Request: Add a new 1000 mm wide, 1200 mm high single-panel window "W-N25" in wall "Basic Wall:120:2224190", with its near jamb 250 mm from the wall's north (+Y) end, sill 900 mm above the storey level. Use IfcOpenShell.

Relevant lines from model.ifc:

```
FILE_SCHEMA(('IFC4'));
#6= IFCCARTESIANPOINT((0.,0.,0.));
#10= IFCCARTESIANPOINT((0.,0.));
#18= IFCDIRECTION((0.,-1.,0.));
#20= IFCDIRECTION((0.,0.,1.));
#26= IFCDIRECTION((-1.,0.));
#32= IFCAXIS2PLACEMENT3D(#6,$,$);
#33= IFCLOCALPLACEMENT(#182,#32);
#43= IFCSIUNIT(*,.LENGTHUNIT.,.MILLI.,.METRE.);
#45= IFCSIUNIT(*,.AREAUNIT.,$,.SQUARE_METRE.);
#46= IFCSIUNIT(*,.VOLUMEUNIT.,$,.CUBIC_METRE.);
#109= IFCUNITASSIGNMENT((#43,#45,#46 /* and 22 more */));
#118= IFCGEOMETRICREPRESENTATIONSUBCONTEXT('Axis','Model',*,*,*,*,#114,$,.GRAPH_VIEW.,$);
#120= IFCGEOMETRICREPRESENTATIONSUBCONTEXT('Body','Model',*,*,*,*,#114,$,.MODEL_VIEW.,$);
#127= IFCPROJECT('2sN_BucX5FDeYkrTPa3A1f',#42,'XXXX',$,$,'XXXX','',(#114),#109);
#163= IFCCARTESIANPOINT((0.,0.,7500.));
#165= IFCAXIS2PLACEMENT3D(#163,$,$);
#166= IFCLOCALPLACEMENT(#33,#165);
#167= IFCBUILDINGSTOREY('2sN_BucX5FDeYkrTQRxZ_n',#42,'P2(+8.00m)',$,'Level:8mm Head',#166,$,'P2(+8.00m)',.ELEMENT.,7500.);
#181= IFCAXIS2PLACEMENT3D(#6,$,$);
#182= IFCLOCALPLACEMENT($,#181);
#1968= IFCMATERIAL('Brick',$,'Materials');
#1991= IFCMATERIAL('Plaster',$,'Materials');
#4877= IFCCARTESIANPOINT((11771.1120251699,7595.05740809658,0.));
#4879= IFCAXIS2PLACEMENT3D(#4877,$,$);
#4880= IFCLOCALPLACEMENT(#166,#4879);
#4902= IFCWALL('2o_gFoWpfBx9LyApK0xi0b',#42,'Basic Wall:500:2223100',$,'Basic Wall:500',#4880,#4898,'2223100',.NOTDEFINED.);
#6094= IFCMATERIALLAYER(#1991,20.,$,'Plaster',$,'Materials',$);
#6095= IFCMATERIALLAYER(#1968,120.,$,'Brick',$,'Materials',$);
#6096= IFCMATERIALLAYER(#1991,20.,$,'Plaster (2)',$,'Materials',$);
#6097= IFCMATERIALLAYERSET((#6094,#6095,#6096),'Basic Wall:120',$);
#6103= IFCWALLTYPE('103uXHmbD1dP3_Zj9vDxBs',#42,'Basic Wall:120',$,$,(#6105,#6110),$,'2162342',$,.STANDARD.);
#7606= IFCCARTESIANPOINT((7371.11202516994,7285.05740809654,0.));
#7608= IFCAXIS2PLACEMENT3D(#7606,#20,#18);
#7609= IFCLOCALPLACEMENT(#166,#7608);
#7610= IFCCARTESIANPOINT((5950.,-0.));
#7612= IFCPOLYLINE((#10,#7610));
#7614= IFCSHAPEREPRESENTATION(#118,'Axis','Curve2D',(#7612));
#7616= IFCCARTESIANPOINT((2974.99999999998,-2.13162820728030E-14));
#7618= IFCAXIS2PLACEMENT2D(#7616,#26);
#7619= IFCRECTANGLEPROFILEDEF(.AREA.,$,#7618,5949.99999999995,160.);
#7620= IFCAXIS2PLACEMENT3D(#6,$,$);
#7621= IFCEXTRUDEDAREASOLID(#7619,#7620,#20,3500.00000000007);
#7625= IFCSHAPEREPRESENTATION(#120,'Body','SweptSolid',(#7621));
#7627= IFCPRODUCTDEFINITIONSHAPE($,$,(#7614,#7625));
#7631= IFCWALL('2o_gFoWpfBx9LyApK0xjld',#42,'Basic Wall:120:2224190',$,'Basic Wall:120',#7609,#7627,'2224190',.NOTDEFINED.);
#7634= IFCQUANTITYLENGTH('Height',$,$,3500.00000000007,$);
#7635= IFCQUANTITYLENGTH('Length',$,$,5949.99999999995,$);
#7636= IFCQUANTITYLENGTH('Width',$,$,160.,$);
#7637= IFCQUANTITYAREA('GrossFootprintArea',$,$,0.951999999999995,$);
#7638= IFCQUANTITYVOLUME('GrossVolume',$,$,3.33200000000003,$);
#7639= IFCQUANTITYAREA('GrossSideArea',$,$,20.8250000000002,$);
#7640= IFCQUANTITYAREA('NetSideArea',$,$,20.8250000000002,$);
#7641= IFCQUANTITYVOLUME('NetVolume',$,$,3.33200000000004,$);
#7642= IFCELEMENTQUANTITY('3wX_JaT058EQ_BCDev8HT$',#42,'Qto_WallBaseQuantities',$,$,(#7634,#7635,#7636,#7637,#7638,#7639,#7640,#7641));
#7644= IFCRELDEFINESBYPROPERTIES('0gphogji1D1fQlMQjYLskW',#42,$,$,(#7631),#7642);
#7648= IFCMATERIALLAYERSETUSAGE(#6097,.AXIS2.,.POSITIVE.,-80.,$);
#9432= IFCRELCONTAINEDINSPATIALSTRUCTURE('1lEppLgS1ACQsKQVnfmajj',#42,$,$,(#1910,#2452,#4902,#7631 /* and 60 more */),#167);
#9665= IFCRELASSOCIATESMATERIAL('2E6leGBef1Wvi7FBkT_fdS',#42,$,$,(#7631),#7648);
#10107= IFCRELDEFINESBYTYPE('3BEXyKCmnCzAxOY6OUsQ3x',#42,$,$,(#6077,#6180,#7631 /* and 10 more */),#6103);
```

```python
import numpy as np
import ifcopenshell
import ifcopenshell.api.feature
import ifcopenshell.api.geometry
import ifcopenshell.api.pset
import ifcopenshell.api.root
import ifcopenshell.api.spatial
import ifcopenshell.geom
import ifcopenshell.util.element
import ifcopenshell.util.placement
import ifcopenshell.util.representation
import ifcopenshell.util.shape
import ifcopenshell.util.unit

model = ifcopenshell.open("model.ifc")
unit_scale = ifcopenshell.util.unit.calculate_unit_scale(model)
area_scale = ifcopenshell.util.unit.calculate_unit_scale(model, "AREAUNIT")
volume_scale = ifcopenshell.util.unit.calculate_unit_scale(model, "VOLUMEUNIT")
settings = ifcopenshell.geom.settings()


def volume(element):
    """Net volume in cubic metres, openings subtracted."""
    shape = ifcopenshell.geom.create_shape(settings, element)
    return ifcopenshell.util.shape.get_volume(shape.geometry)


wall = model.by_guid("2o_gFoWpfBx9LyApK0xjld")
storey = ifcopenshell.util.element.get_container(wall, ifc_class="IfcBuildingStorey")
context = ifcopenshell.util.representation.get_context(model, "Model", "Body", "MODEL_VIEW")
before = volume(wall)

width, height, from_end, sill = 1, 1.2, 0.25, 0.9  # metres

# The wall runs along its own X axis, and the end named is its -X end.
wall_shape = ifcopenshell.geom.create_shape(settings, wall)
x, y, z = ifcopenshell.util.shape.get_vertices(wall_shape.geometry).T
start = x.min() + from_end
face, thickness = float(y.min()), float(y.max() - y.min())
wall_matrix = ifcopenshell.util.placement.get_local_placement(wall.ObjectPlacement)
level = ifcopenshell.util.placement.get_local_placement(storey.ObjectPlacement)[2, 3]


def in_wall(x, y):
    """Placement at x, y metres in the wall's axes, at sill height."""
    matrix = wall_matrix.copy()
    matrix[:, 3] = wall_matrix @ np.array([x / unit_scale, y / unit_scale, 0.0, 1.0])
    matrix[2, 3] = level + sill / unit_scale
    return matrix


# Opening: a box that overshoots both wall faces by 50 mm.
opening = ifcopenshell.api.root.create_entity(model, ifc_class="IfcOpeningElement", predefined_type="OPENING")
box = ifcopenshell.api.geometry.add_wall_representation(
    model, context=context, length=width, height=height, thickness=thickness + 0.1
)
ifcopenshell.api.geometry.assign_representation(model, product=opening, representation=box)
ifcopenshell.api.geometry.edit_object_placement(model, product=opening, matrix=in_wall(start, face - 0.05), is_si=False)
ifcopenshell.api.feature.add_feature(model, feature=opening, element=wall)

window = ifcopenshell.api.root.create_entity(model, ifc_class="IfcWindow", name="W-N25", predefined_type="WINDOW")
window.OverallWidth, window.OverallHeight = width / unit_scale, height / unit_scale
window.PartitioningType = "SINGLE_PANEL"
body = ifcopenshell.api.geometry.add_window_representation(
    model,
    context=context,
    overall_width=window.OverallWidth,
    overall_height=window.OverallHeight,
    partition_type="SINGLE_PANEL",
)
ifcopenshell.api.geometry.assign_representation(model, product=window, representation=body)
ifcopenshell.api.spatial.assign_container(model, products=[window], relating_structure=storey)
ifcopenshell.api.feature.add_filling(model, opening=opening, element=window)

# Centre the window in the wall's thickness.
ifcopenshell.api.geometry.edit_object_placement(model, product=window, matrix=in_wall(start, face), is_si=False)
window_shape = ifcopenshell.geom.create_shape(settings, window)
depth = ifcopenshell.util.shape.get_vertices(window_shape.geometry)[:, 1]
offset = face + thickness / 2 - (depth.min() + depth.max()) / 2
ifcopenshell.api.geometry.edit_object_placement(model, product=window, matrix=in_wall(start, offset), is_si=False)

after = volume(wall)

# Update the wall's stored quantities.
qto = model.by_id(ifcopenshell.util.element.get_pset(wall, "Qto_WallBaseQuantities", should_inherit=False)["id"])
ifcopenshell.api.pset.edit_qto(model, qto=qto, properties={
    "NetSideArea": after / thickness / area_scale,
    "NetVolume": after / volume_scale,
})

print(f"wall volume {before:.3f} -> {after:.3f} m3")

model.write("model_v2.ifc")
```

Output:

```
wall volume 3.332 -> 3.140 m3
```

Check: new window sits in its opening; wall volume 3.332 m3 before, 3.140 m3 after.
